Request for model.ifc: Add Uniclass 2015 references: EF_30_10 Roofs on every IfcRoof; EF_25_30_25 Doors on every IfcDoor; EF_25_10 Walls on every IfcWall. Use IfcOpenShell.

First a look at what the model holds.

```python
import ifcopenshell

model = ifcopenshell.open("model.ifc")
print(model.schema)
print("classifications:", [c.Name for c in model.by_type("IfcClassification")])
for ifc_class in ("IfcDoor", "IfcRoof", "IfcStair", "IfcWall", "IfcWindow"):
    print(ifc_class, len(model.by_type(ifc_class)))
```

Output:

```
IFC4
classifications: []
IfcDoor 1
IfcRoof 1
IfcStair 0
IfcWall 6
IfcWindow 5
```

```python
import ifcopenshell
import ifcopenshell.api.classification

model = ifcopenshell.open("model.ifc")

system = ifcopenshell.api.classification.add_classification(model, classification="Uniclass 2015")

codes = {
    "IfcRoof": ("EF_30_10", "Roofs"),
    "IfcDoor": ("EF_25_30_25", "Doors"),
    "IfcWall": ("EF_25_10", "Walls"),
}
for ifc_class, (code, name) in codes.items():
    products = model.by_type(ifc_class)
    ifcopenshell.api.classification.add_reference(
        model, products=products, classification=system, identification=code, name=name
    )
    print(code, len(products))

model.write("model_updated.ifc")
```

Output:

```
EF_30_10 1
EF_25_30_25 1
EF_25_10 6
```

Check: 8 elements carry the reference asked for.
